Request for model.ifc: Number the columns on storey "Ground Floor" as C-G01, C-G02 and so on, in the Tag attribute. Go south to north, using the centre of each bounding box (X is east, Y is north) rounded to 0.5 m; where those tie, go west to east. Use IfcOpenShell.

First a look at what the model holds.

```python
import ifcopenshell
import ifcopenshell.util.element
import ifcopenshell.util.placement

model = ifcopenshell.open("model.ifc")
print(model.schema)
storey = next(s for s in model.by_type("IfcBuildingStorey") if s.Name == "Ground Floor")
columns = [e for e in ifcopenshell.util.element.get_decomposition(storey) if e.is_a("IfcColumn")]
for e in sorted(columns, key=lambda e: e.id()):
    origin = ifcopenshell.util.placement.get_local_placement(e.ObjectPlacement)[:3, 3]
    print(e.id(), e.Tag, e.Name, origin.round(2) + 0.0, sep=" | ")
```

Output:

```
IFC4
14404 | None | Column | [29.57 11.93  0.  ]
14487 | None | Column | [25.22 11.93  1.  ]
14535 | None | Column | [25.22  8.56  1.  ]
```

```python
import ifcopenshell
import ifcopenshell.geom
import ifcopenshell.util.element
import ifcopenshell.util.shape

model = ifcopenshell.open("model.ifc")
settings = ifcopenshell.geom.settings()
settings.set("use-world-coords", True)


def centre(element):
    shape = ifcopenshell.geom.create_shape(settings, element)
    return ifcopenshell.util.shape.get_bbox_centroid(shape.geometry)


storey = next(s for s in model.by_type("IfcBuildingStorey") if s.Name == "Ground Floor")
columns = [e for e in ifcopenshell.util.element.get_decomposition(storey) if e.is_a("IfcColumn")]

# Insertion points can sit at a corner or the storey origin, so sort by the geometry (in metres).
centres = {e: centre(e) for e in columns}
columns.sort(key=lambda e: (round(centres[e][1] / 0.5), centres[e][0]))

for i, e in enumerate(columns, start=1):
    number = f"C-G{i:02d}"
    e.Tag = number
    print(e.id(), number)

model.write("model_edited.ifc")
```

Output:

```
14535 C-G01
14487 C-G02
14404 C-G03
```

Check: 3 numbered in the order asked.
